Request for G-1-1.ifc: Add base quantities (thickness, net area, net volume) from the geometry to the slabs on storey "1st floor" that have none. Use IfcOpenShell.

First a look at what the model holds.

```python
import ifcopenshell
import ifcopenshell.util.element
import ifcopenshell.util.unit

model = ifcopenshell.open("G-1-1.ifc")
print(model.schema)
for unit_type in ("LENGTHUNIT", "AREAUNIT", "VOLUMEUNIT"):
    print(unit_type, ifcopenshell.util.unit.calculate_unit_scale(model, unit_type))
storey = next(s for s in model.by_type("IfcBuildingStorey") if s.Name == "1st floor")
slabs = [e for e in ifcopenshell.util.element.get_decomposition(storey) if e.is_a("IfcSlab")]
for e in sorted(slabs, key=lambda e: e.id()):
    print(e.id(), e.is_a(), e.Name, list(ifcopenshell.util.element.get_psets(e, qtos_only=True)), sep=" | ")
```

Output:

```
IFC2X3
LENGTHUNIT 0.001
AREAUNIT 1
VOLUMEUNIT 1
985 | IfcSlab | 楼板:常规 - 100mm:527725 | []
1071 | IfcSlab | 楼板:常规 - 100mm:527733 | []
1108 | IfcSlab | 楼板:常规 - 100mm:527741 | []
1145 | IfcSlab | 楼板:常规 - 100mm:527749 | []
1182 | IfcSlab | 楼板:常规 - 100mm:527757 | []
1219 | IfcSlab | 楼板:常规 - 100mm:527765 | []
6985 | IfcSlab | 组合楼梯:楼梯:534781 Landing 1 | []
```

```python
import ifcopenshell
import ifcopenshell.api.pset
import ifcopenshell.geom
import ifcopenshell.util.element
import ifcopenshell.util.shape
import ifcopenshell.util.unit

model = ifcopenshell.open("G-1-1.ifc")
unit_scale = ifcopenshell.util.unit.calculate_unit_scale(model)
area_scale = ifcopenshell.util.unit.calculate_unit_scale(model, "AREAUNIT")
volume_scale = ifcopenshell.util.unit.calculate_unit_scale(model, "VOLUMEUNIT")
settings = ifcopenshell.geom.settings()

storey = next(s for s in model.by_type("IfcBuildingStorey") if s.Name == "1st floor")
slabs = [e for e in ifcopenshell.util.element.get_decomposition(storey) if e.is_a("IfcSlab")]

for e in sorted(slabs, key=lambda e: e.id()):
    if ifcopenshell.util.element.get_psets(e, qtos_only=True, should_inherit=False):
        continue
    # Geometry comes back in metres, in the element's own axes.
    shape = ifcopenshell.geom.create_shape(settings, e)
    values = {
        "Width": ifcopenshell.util.shape.get_z(shape.geometry) / unit_scale,
        "NetArea": ifcopenshell.util.shape.get_footprint_area(shape.geometry) / area_scale,
        "NetVolume": ifcopenshell.util.shape.get_volume(shape.geometry) / volume_scale,
    }
    qto = ifcopenshell.api.pset.add_qto(model, product=e, name="BaseQuantities")
    ifcopenshell.api.pset.edit_qto(model, qto=qto, properties=values)
    print(e.id(), {k: round(v, 3) for k, v in values.items()})

model.write("G-1-1_v2.ifc")
```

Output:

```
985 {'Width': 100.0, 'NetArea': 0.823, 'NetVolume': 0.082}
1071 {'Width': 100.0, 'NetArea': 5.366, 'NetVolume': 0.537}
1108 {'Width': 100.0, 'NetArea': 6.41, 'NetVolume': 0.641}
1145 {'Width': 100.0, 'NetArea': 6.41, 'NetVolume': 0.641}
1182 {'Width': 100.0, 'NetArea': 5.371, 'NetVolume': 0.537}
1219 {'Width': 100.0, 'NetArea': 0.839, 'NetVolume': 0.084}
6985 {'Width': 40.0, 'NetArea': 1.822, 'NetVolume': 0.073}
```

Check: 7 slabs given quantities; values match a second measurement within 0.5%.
